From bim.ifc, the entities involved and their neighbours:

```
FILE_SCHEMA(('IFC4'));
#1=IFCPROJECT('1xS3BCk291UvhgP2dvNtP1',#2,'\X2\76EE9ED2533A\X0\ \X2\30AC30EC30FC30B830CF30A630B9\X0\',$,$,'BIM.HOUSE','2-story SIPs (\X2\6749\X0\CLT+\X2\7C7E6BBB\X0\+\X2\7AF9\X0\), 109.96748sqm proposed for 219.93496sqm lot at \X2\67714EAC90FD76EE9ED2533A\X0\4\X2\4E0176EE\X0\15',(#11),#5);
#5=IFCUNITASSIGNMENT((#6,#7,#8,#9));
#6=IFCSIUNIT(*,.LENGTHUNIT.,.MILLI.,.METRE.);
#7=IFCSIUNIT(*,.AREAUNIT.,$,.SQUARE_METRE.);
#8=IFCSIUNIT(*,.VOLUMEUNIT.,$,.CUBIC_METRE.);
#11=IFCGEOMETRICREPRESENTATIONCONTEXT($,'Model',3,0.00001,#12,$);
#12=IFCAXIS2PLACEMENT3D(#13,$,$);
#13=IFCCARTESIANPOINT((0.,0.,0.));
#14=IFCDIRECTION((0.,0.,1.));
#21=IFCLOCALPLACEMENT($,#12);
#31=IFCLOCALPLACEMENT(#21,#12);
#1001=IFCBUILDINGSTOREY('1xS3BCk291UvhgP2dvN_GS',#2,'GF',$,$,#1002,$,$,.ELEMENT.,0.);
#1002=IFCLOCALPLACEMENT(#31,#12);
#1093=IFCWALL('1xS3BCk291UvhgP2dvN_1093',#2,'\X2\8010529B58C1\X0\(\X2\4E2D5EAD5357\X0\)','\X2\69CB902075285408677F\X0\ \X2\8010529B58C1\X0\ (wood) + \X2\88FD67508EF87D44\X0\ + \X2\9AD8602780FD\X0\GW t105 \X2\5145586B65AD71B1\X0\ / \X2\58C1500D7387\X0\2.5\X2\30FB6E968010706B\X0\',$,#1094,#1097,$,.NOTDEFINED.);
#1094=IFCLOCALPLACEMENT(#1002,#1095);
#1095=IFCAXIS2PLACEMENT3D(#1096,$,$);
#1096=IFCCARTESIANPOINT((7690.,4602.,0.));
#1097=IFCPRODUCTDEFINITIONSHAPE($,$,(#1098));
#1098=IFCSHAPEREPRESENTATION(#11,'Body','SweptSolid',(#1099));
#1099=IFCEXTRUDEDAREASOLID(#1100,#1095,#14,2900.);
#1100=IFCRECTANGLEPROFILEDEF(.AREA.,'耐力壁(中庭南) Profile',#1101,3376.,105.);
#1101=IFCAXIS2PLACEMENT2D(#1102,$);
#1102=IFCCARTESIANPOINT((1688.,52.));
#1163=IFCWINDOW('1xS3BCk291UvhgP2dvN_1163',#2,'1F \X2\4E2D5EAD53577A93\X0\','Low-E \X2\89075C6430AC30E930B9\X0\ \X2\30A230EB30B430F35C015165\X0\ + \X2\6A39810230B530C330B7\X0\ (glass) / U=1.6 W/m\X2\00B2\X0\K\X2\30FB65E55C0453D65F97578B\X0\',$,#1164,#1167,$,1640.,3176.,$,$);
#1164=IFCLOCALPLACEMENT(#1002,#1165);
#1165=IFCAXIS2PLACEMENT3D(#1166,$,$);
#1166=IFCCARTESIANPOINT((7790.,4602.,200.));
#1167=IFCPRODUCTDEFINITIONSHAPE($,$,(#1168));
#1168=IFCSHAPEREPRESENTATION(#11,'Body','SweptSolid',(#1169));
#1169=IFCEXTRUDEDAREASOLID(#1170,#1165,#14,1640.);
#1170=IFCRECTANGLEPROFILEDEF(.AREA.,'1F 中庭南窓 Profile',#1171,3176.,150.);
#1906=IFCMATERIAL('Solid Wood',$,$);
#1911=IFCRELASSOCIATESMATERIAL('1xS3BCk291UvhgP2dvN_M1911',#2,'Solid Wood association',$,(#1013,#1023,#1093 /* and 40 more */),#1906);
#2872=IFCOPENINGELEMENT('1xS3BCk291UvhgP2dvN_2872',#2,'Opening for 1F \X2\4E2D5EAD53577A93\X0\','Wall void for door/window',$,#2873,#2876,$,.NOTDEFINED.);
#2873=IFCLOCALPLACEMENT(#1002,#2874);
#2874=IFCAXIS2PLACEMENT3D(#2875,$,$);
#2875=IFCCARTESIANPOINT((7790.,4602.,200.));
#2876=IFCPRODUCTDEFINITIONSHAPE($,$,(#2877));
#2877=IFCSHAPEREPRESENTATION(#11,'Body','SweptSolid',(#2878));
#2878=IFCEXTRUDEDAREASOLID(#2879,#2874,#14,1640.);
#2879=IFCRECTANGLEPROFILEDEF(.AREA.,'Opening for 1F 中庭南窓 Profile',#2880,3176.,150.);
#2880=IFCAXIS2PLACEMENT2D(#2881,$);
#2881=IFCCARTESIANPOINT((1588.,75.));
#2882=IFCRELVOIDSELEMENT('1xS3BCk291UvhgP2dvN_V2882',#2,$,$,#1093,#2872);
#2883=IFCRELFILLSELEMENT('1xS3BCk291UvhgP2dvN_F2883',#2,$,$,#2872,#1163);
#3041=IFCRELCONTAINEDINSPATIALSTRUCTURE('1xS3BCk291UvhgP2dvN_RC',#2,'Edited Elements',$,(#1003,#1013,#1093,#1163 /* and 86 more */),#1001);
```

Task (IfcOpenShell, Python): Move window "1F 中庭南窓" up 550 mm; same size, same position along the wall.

```python
import numpy as np
import ifcopenshell
import ifcopenshell.api.geometry
import ifcopenshell.util.placement
import ifcopenshell.util.unit

model = ifcopenshell.open("bim.ifc")
unit_scale = ifcopenshell.util.unit.calculate_unit_scale(model)

window = model.by_guid("1xS3BCk291UvhgP2dvN_1163")
opening = window.FillsVoids[0].RelatingOpeningElement
dz = 550.0

shift = np.array([0.0, 0.0, dz])
# The window is not placed relative to its opening, so move both.
for product in (opening, window):
    matrix = ifcopenshell.util.placement.get_local_placement(product.ObjectPlacement)
    matrix[:3, 3] += shift
    ifcopenshell.api.geometry.edit_object_placement(model, product=product, matrix=matrix, is_si=False)

print(f"moved by {dz * unit_scale:+.3f} m")

model.write("bim_rev.ifc")
```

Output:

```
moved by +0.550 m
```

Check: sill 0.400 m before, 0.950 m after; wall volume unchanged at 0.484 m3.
